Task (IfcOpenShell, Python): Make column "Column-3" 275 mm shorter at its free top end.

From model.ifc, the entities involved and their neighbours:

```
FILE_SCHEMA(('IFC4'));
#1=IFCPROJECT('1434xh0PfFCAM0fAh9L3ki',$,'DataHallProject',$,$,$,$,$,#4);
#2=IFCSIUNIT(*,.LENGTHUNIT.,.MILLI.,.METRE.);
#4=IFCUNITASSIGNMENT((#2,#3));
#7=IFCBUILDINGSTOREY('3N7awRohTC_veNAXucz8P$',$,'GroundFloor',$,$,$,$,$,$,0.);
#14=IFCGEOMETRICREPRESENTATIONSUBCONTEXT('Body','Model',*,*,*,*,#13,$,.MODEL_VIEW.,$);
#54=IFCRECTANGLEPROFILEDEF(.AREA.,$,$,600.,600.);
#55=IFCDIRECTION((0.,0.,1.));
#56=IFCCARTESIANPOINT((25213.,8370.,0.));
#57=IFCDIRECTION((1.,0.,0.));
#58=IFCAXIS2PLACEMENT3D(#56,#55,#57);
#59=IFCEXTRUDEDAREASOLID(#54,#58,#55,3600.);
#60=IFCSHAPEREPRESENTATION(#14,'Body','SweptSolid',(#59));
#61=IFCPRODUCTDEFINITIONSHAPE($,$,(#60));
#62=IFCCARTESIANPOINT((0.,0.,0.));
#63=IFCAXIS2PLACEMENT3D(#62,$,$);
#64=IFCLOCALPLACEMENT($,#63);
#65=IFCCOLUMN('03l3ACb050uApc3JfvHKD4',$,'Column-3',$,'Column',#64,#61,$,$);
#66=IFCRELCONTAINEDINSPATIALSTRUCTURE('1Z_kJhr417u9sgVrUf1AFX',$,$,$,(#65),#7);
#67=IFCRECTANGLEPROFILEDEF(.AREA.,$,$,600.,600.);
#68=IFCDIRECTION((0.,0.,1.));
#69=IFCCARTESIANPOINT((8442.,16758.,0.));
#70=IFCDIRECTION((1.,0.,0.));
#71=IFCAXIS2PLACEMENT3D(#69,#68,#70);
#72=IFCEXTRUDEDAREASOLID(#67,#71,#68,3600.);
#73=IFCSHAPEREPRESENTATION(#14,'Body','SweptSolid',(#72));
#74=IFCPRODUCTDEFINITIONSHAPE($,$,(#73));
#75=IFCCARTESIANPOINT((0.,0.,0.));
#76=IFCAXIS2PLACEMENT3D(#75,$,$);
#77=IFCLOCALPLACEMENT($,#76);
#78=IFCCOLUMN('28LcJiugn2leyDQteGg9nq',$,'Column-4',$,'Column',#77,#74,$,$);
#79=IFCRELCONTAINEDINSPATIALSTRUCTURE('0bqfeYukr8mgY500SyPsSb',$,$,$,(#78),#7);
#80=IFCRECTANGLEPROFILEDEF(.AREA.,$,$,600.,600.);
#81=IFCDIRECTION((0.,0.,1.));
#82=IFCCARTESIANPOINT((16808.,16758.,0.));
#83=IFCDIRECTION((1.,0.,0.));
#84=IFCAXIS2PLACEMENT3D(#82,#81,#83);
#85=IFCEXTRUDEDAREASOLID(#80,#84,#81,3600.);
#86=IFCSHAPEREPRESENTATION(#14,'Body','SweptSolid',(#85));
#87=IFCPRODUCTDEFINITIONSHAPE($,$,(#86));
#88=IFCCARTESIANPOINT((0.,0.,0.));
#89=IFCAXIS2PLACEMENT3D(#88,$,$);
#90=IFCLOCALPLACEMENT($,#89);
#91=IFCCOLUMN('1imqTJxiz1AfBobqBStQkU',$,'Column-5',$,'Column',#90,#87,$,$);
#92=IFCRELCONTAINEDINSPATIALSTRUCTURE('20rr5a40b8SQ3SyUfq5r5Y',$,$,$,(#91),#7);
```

```python
import ifcopenshell
import ifcopenshell.util.representation
import ifcopenshell.util.unit

model = ifcopenshell.open("model.ifc")
unit_scale = ifcopenshell.util.unit.calculate_unit_scale(model)

member = model.by_guid("03l3ACb050uApc3JfvHKD4")
change = -0.275 / unit_scale

# The extrusion runs towards the end named, so only its depth changes.
body = ifcopenshell.util.representation.get_representation(member, "Model", "Body")
solid = body.Items[0]
old_length = solid.Depth
solid.Depth += change

print(f"length {old_length:g} -> {solid.Depth:g}")

model.write("model_v2.ifc")
```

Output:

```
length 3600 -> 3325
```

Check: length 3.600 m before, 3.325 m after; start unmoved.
